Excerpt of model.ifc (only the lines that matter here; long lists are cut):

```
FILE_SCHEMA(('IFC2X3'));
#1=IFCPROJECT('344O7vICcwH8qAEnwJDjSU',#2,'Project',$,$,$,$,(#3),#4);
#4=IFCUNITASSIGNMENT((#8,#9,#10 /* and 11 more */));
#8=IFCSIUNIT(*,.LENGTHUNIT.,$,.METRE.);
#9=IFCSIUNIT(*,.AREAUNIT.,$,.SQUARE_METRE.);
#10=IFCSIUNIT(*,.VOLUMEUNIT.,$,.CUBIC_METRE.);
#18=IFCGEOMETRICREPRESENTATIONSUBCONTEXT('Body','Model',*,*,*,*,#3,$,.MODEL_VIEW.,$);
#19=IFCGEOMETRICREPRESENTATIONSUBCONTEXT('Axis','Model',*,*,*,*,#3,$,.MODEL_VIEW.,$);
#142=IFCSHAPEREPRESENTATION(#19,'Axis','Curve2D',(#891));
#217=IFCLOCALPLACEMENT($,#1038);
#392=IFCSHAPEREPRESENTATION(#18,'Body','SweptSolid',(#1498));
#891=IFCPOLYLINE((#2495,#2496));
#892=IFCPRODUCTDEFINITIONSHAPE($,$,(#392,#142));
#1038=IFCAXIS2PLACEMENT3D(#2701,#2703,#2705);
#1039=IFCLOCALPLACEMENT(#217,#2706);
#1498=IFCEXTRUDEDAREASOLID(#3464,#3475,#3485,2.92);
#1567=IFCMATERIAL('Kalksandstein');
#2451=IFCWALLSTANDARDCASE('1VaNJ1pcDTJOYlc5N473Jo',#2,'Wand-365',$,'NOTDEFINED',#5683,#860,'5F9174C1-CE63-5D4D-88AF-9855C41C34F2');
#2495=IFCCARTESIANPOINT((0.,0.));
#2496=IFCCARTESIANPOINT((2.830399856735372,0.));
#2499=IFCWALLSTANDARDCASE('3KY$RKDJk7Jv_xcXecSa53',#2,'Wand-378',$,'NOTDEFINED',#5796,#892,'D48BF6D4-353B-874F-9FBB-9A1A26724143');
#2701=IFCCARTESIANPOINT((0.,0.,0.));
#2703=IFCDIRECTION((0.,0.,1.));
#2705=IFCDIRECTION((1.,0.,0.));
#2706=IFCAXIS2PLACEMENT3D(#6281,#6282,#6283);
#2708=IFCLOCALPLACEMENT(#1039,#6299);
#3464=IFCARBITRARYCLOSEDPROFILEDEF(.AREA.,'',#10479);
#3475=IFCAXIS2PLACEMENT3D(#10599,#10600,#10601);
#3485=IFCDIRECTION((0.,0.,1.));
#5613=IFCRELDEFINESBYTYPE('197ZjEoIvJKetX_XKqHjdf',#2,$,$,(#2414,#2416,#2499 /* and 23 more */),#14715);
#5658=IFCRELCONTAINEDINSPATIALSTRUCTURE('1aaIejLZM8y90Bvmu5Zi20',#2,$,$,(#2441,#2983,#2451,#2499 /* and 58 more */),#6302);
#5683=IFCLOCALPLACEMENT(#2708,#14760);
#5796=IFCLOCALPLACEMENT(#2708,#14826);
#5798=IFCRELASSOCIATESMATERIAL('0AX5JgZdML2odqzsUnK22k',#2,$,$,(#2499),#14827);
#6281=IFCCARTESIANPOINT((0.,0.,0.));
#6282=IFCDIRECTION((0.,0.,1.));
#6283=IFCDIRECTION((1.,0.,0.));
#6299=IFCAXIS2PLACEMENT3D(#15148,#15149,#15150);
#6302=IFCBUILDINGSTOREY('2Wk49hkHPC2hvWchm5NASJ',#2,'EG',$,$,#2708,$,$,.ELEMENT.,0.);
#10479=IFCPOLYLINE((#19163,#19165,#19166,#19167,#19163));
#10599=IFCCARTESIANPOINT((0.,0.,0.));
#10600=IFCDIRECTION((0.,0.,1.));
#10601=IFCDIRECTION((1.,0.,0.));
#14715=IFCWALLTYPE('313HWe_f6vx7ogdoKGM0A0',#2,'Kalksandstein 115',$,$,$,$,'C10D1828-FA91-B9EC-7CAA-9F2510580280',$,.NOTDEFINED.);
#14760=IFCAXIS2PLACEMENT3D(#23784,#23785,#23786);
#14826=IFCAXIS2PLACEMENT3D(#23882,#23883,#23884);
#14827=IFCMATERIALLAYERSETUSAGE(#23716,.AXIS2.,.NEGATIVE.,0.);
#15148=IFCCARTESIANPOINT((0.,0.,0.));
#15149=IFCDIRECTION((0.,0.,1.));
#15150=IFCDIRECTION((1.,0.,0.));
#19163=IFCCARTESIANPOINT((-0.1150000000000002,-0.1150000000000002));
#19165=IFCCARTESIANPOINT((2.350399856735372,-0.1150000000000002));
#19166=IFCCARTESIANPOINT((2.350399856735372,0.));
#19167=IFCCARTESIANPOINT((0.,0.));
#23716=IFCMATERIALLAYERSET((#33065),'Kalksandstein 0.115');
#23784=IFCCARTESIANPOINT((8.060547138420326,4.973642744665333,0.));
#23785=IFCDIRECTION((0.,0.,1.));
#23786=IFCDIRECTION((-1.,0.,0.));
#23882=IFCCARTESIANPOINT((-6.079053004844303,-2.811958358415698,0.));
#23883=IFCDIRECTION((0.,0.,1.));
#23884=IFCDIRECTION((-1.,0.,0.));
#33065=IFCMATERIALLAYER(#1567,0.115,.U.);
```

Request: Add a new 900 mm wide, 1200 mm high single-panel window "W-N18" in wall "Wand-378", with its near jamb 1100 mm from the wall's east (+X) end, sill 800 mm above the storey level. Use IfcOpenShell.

```python
import numpy as np
import ifcopenshell
import ifcopenshell.api.feature
import ifcopenshell.api.geometry
import ifcopenshell.api.root
import ifcopenshell.api.spatial
import ifcopenshell.api.type
import ifcopenshell.geom
import ifcopenshell.util.element
import ifcopenshell.util.placement
import ifcopenshell.util.representation
import ifcopenshell.util.shape
import ifcopenshell.util.unit

model = ifcopenshell.open("model.ifc")
unit_scale = ifcopenshell.util.unit.calculate_unit_scale(model)
settings = ifcopenshell.geom.settings()


def volume(element):
    """Net volume in cubic metres, openings subtracted."""
    shape = ifcopenshell.geom.create_shape(settings, element)
    return ifcopenshell.util.shape.get_volume(shape.geometry)


wall = model.by_guid("3KY$RKDJk7Jv_xcXecSa53")
storey = ifcopenshell.util.element.get_container(wall, ifc_class="IfcBuildingStorey")
context = ifcopenshell.util.representation.get_context(model, "Model", "Body", "MODEL_VIEW")
before = volume(wall)

width, height, from_end, sill = 0.9, 1.2, 1.1, 0.8  # metres

# The wall runs along its own X axis, and the end named is its -X end.
wall_shape = ifcopenshell.geom.create_shape(settings, wall)
x, y, z = ifcopenshell.util.shape.get_vertices(wall_shape.geometry).T
start = x.min() + from_end
face, thickness = float(y.min()), float(y.max() - y.min())
wall_matrix = ifcopenshell.util.placement.get_local_placement(wall.ObjectPlacement)
level = ifcopenshell.util.placement.get_local_placement(storey.ObjectPlacement)[2, 3]


def in_wall(x, y):
    """Placement at x, y metres in the wall's axes, at sill height."""
    matrix = wall_matrix.copy()
    matrix[:, 3] = wall_matrix @ np.array([x / unit_scale, y / unit_scale, 0.0, 1.0])
    matrix[2, 3] = level + sill / unit_scale
    return matrix


# Opening: a box that overshoots both wall faces by 50 mm.
opening = ifcopenshell.api.root.create_entity(model, ifc_class="IfcOpeningElement")
box = ifcopenshell.api.geometry.add_wall_representation(
    model, context=context, length=width, height=height, thickness=thickness + 0.1
)
ifcopenshell.api.geometry.assign_representation(model, product=opening, representation=box)
ifcopenshell.api.geometry.edit_object_placement(model, product=opening, matrix=in_wall(start, face - 0.05), is_si=False)
ifcopenshell.api.feature.add_feature(model, feature=opening, element=wall)

window = ifcopenshell.api.root.create_entity(model, ifc_class="IfcWindow", name="W-N18")
window.OverallWidth, window.OverallHeight = width / unit_scale, height / unit_scale
body = ifcopenshell.api.geometry.add_window_representation(
    model,
    context=context,
    overall_width=window.OverallWidth,
    overall_height=window.OverallHeight,
    partition_type="SINGLE_PANEL",
)
ifcopenshell.api.geometry.assign_representation(model, product=window, representation=body)
ifcopenshell.api.spatial.assign_container(model, products=[window], relating_structure=storey)
fills = ifcopenshell.api.feature.add_filling(model, opening=opening, element=window)
fills.OwnerHistory = window.OwnerHistory  # required in IFC2X3

# IFC2X3 keeps the operation on the window style.
style = ifcopenshell.api.root.create_entity(model, ifc_class="IfcWindowStyle", name="W-N18")
style.OperationType, style.ConstructionType = "SINGLE_PANEL", "NOTDEFINED"
style.ParameterTakesPrecedence = style.Sizeable = False
ifcopenshell.api.type.assign_type(model, related_objects=[window], relating_type=style)

# Centre the window in the wall's thickness.
ifcopenshell.api.geometry.edit_object_placement(model, product=window, matrix=in_wall(start, face), is_si=False)
window_shape = ifcopenshell.geom.create_shape(settings, window)
depth = ifcopenshell.util.shape.get_vertices(window_shape.geometry)[:, 1]
offset = face + thickness / 2 - (depth.min() + depth.max()) / 2
ifcopenshell.api.geometry.edit_object_placement(model, product=window, matrix=in_wall(start, offset), is_si=False)

after = volume(wall)

print(f"wall volume {before:.3f} -> {after:.3f} m3")

model.write("model_updated.ifc")
```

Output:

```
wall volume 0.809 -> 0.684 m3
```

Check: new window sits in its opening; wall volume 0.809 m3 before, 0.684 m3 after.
